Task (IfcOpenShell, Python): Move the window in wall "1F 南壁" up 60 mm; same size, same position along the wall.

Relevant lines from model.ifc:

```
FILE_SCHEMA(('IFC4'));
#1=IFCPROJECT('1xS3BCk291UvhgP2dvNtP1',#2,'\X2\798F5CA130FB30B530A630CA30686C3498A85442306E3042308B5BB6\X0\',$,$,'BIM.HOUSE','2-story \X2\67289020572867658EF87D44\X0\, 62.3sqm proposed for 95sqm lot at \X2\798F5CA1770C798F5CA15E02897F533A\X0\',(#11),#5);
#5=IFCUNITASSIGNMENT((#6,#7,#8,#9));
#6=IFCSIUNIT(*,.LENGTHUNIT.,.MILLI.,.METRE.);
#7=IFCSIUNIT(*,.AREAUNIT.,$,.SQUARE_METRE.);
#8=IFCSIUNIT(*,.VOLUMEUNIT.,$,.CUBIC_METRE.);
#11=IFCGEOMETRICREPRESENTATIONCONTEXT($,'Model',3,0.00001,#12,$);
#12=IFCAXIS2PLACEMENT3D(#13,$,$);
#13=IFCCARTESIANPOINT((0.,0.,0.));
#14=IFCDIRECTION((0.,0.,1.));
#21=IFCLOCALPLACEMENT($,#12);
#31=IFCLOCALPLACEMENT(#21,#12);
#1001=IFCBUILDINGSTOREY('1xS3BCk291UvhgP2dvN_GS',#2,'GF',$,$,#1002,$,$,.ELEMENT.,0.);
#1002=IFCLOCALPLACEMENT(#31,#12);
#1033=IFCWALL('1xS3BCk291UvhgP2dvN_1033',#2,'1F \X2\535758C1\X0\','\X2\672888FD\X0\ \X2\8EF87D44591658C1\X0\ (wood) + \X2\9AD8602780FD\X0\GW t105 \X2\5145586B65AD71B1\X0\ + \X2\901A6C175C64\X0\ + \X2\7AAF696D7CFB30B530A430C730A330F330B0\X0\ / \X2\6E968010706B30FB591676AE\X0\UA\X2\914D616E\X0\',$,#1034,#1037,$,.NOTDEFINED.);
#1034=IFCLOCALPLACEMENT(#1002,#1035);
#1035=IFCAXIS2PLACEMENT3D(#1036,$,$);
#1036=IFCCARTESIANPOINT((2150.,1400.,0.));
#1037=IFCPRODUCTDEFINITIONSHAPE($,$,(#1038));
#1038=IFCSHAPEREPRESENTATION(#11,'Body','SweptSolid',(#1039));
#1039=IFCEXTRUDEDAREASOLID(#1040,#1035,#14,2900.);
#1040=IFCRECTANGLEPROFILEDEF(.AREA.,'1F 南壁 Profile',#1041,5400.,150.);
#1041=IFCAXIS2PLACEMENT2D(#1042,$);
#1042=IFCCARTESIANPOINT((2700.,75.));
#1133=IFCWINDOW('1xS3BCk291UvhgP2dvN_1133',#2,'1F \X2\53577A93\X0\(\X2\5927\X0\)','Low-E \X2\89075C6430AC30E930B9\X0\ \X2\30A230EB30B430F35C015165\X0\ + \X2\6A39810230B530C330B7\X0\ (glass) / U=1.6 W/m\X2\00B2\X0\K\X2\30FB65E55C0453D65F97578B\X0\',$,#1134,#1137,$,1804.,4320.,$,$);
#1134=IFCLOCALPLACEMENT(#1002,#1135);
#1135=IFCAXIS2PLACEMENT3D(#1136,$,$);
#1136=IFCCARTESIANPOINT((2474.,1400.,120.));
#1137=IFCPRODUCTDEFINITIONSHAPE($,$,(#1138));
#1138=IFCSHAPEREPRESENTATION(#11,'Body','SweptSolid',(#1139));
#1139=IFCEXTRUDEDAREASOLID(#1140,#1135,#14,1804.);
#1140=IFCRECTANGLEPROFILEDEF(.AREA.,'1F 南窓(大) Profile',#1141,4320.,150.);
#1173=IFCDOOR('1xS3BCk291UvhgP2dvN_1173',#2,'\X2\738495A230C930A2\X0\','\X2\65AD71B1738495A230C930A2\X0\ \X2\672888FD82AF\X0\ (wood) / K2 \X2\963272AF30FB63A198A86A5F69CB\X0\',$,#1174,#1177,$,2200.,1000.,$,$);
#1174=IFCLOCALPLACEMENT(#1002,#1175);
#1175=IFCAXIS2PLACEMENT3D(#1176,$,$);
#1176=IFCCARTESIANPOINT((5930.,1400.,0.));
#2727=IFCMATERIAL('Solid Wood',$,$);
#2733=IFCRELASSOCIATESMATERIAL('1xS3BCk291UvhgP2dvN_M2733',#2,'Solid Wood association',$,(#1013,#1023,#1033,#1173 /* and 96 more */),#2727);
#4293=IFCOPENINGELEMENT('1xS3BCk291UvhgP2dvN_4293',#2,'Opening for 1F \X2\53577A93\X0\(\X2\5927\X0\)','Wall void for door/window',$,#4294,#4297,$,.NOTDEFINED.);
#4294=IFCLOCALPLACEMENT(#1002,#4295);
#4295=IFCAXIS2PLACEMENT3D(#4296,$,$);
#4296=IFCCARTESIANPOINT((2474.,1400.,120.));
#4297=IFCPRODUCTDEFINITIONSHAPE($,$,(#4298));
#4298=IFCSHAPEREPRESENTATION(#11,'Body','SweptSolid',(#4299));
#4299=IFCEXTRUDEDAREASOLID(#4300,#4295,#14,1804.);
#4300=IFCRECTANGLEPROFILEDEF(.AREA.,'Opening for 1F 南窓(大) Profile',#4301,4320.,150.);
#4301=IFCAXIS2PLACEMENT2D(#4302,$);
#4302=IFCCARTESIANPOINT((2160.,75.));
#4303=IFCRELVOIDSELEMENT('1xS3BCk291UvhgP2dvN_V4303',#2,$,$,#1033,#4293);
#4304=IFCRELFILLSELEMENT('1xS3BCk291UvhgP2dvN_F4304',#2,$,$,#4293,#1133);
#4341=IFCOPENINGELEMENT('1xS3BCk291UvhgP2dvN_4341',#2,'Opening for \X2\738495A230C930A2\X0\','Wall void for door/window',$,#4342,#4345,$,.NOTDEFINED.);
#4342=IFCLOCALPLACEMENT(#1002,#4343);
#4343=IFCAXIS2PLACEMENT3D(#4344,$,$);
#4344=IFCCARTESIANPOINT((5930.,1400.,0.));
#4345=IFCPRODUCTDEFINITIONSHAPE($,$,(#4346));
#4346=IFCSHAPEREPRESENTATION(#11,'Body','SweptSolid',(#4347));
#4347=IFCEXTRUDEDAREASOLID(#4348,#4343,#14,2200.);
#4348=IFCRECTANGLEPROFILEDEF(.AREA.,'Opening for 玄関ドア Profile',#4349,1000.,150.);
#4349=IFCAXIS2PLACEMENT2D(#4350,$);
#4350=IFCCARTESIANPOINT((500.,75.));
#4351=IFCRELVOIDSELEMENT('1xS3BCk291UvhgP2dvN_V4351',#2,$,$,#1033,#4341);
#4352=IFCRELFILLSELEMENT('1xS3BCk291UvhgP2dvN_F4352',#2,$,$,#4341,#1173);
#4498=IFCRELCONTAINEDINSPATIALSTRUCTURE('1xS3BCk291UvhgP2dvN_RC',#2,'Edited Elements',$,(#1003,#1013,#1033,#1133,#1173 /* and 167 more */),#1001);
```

```python
import numpy as np
import ifcopenshell
import ifcopenshell.api.geometry
import ifcopenshell.util.placement
import ifcopenshell.util.unit

model = ifcopenshell.open("model.ifc")
unit_scale = ifcopenshell.util.unit.calculate_unit_scale(model)

window = model.by_id(1133)
opening = window.FillsVoids[0].RelatingOpeningElement
dz = 60.0

shift = np.array([0.0, 0.0, dz])
# The window is not placed relative to its opening, so move both.
for product in (opening, window):
    matrix = ifcopenshell.util.placement.get_local_placement(product.ObjectPlacement)
    matrix[:3, 3] += shift
    ifcopenshell.api.geometry.edit_object_placement(model, product=product, matrix=matrix, is_si=False)

print(f"moved by {dz * unit_scale:+.3f} m")

model.write("model_rev.ifc")
```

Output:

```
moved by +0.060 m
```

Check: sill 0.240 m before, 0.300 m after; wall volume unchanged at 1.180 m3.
